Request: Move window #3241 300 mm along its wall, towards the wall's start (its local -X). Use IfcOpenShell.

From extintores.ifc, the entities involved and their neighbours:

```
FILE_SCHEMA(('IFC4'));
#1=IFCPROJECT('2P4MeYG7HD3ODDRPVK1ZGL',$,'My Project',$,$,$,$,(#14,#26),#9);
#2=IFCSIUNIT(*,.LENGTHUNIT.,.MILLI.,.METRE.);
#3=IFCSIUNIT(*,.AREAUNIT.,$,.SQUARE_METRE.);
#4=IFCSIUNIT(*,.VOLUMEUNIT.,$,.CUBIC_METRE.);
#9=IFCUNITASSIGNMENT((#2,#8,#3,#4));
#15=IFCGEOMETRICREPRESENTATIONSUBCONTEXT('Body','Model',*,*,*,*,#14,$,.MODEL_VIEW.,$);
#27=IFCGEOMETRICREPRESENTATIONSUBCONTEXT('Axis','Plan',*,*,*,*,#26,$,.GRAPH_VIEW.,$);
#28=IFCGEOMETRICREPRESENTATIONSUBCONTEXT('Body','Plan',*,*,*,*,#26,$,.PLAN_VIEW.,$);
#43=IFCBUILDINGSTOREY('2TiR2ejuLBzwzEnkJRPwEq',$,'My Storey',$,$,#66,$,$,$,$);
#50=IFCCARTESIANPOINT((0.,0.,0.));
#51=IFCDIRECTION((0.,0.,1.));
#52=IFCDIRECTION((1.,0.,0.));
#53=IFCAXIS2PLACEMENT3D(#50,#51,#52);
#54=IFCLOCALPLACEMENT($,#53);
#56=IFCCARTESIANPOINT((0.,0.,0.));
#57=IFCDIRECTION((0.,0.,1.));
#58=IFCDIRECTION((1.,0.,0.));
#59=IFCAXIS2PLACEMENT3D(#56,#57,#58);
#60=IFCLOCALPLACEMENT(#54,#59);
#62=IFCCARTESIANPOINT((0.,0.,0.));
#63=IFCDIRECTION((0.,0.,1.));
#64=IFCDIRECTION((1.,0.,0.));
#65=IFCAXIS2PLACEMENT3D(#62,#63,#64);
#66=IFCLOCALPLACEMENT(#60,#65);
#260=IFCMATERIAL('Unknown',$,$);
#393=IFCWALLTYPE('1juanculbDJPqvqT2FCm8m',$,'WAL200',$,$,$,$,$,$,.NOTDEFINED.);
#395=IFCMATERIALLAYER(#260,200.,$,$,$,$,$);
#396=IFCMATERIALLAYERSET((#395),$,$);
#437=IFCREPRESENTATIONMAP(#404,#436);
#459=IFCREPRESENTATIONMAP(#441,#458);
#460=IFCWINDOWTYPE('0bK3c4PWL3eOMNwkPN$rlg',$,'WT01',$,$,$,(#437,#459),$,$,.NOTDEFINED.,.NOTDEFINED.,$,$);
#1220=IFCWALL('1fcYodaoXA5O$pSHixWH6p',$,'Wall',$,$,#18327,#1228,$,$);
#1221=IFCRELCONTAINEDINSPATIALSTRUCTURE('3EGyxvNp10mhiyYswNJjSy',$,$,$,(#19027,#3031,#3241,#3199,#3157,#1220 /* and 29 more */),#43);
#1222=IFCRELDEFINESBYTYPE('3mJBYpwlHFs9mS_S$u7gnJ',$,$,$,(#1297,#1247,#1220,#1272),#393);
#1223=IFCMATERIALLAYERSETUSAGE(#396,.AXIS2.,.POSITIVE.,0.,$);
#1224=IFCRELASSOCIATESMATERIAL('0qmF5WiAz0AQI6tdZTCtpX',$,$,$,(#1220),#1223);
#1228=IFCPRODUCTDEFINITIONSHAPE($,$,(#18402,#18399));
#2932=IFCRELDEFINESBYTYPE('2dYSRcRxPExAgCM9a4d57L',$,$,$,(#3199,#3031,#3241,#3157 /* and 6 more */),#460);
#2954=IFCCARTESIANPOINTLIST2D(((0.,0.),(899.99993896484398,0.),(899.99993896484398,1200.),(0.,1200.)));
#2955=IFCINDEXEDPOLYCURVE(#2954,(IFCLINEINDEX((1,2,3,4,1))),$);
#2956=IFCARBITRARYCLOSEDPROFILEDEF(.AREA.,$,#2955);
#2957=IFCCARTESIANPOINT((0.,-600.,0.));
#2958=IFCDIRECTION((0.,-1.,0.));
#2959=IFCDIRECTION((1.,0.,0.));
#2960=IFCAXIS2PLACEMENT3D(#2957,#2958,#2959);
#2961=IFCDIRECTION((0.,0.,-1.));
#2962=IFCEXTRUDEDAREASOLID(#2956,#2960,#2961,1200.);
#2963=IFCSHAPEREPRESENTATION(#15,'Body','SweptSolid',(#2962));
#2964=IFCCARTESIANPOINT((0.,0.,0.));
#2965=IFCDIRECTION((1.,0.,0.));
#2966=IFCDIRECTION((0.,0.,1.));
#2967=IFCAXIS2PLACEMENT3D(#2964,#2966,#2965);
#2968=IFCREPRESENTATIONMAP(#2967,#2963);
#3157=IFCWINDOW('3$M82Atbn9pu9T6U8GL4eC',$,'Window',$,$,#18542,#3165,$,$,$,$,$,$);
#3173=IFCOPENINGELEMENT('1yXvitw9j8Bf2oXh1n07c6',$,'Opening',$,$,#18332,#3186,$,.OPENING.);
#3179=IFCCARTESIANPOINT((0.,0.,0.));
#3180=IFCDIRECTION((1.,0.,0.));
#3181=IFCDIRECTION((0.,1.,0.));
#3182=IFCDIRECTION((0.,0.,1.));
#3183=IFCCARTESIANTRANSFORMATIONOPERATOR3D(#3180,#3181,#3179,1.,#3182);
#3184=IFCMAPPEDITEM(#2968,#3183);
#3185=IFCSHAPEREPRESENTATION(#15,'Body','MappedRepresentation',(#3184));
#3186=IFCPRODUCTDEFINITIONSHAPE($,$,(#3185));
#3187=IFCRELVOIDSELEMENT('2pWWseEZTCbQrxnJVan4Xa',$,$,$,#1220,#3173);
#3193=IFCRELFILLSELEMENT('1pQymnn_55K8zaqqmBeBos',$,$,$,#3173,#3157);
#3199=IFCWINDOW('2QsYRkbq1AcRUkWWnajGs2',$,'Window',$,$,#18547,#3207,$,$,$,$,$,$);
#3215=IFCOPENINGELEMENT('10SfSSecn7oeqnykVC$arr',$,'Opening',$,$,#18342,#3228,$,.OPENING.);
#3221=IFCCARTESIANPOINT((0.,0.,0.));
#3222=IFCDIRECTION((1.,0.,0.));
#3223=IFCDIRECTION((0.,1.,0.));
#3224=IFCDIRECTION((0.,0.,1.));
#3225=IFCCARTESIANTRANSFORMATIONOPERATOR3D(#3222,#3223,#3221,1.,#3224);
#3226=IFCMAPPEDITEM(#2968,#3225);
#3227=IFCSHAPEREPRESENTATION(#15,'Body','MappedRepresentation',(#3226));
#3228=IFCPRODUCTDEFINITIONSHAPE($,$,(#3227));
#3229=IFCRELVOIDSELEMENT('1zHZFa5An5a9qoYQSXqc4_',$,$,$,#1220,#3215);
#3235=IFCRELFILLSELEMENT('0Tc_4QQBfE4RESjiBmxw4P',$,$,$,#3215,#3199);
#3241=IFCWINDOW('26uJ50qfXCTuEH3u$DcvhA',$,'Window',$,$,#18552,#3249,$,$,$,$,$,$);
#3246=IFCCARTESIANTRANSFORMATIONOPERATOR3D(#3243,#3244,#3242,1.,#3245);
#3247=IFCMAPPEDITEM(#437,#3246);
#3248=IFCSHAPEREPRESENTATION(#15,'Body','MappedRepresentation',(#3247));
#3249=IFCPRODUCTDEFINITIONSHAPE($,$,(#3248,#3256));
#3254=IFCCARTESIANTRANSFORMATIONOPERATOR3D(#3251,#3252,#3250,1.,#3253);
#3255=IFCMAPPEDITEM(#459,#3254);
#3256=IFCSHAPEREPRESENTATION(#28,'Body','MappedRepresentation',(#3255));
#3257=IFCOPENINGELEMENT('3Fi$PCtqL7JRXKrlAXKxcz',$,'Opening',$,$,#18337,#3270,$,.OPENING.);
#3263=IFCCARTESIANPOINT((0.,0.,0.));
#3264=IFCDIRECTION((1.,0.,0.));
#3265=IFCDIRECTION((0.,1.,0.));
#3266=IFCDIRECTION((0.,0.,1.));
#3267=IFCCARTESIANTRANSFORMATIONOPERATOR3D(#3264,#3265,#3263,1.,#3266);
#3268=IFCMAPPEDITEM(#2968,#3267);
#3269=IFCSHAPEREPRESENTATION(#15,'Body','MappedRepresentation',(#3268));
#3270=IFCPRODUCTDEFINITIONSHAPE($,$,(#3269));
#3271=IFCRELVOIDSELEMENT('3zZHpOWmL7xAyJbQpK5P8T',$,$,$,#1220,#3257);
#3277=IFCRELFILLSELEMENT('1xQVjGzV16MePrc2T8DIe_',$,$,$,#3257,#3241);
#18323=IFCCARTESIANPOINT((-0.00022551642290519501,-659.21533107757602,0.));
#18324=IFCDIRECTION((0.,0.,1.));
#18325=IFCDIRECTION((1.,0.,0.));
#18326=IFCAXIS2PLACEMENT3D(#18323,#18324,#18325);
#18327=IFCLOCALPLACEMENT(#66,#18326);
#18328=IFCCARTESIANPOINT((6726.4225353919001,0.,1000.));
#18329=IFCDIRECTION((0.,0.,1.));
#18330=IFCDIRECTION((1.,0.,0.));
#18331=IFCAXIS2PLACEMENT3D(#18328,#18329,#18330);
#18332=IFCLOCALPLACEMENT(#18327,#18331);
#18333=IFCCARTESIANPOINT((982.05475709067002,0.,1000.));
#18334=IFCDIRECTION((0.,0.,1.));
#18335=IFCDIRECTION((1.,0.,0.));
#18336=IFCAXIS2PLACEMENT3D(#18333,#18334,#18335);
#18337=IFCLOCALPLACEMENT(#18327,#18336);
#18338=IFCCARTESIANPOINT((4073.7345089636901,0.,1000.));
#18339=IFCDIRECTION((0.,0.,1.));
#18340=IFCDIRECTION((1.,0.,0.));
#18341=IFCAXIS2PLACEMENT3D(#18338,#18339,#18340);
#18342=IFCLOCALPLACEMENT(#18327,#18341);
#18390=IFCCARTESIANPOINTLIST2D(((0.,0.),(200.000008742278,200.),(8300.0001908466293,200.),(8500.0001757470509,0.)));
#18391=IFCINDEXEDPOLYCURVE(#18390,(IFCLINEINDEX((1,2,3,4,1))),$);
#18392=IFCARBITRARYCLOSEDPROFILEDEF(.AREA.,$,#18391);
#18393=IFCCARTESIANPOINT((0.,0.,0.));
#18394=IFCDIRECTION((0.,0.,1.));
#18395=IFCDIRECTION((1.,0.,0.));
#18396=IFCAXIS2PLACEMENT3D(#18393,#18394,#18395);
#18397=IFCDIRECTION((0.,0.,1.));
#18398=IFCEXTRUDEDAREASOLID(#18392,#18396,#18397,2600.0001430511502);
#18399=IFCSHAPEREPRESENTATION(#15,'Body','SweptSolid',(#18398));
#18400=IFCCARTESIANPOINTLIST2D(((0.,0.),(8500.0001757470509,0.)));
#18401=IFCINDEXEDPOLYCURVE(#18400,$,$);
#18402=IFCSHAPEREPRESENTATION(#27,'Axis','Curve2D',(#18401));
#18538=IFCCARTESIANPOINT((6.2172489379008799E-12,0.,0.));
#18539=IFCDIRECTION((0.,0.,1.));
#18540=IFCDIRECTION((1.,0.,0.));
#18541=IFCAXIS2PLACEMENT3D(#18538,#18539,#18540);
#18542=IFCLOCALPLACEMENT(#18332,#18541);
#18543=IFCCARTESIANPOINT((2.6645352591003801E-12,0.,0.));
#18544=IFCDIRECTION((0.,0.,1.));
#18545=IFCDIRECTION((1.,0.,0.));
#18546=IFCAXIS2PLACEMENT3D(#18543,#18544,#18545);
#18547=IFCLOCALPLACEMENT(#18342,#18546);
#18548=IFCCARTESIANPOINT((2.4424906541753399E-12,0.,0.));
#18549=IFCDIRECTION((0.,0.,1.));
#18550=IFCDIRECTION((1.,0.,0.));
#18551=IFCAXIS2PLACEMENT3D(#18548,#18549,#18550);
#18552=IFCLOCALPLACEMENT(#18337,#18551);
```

```python
import ifcopenshell
import ifcopenshell.api.geometry
import ifcopenshell.util.placement
import ifcopenshell.util.unit

model = ifcopenshell.open("extintores.ifc")
unit_scale = ifcopenshell.util.unit.calculate_unit_scale(model)

window = model.by_id(3241)
opening = window.FillsVoids[0].RelatingOpeningElement
wall = opening.VoidsElements[0].RelatingBuildingElement

wall_matrix = ifcopenshell.util.placement.get_local_placement(wall.ObjectPlacement)
shift = wall_matrix[:3, 0] * -0.3 / unit_scale
before = ifcopenshell.util.placement.get_local_placement(window.ObjectPlacement)[:3, 3].copy()

# The window is placed relative to its opening, so it follows when the opening moves.
matrix = ifcopenshell.util.placement.get_local_placement(opening.ObjectPlacement)
matrix[:3, 3] += shift
ifcopenshell.api.geometry.edit_object_placement(
    model, product=opening, matrix=matrix, is_si=False, should_transform_children=True
)

after = ifcopenshell.util.placement.get_local_placement(window.ObjectPlacement)[:3, 3]
print("window moved by", (after - before).round(3) + 0.0)

model.write("extintores-out.ifc")
```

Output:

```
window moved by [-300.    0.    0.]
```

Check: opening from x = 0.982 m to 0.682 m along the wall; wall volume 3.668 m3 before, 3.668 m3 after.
